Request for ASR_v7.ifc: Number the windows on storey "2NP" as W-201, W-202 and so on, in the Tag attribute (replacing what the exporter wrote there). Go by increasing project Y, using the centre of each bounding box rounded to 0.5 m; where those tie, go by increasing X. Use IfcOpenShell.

First a look at what the model holds.

```python
import ifcopenshell
import ifcopenshell.util.element
import ifcopenshell.util.placement

model = ifcopenshell.open("ASR_v7.ifc")
print(model.schema)
storey = next(s for s in model.by_type("IfcBuildingStorey") if s.Name == "2NP")
windows = [e for e in ifcopenshell.util.element.get_decomposition(storey) if e.is_a("IfcWindow")]
for e in sorted(windows, key=lambda e: e.id()):
    origin = ifcopenshell.util.placement.get_local_placement(e.ObjectPlacement)[:3, 3]
    print(e.id(), e.Tag, e.Name, origin.round(2) + 0.0, sep=" | ")
```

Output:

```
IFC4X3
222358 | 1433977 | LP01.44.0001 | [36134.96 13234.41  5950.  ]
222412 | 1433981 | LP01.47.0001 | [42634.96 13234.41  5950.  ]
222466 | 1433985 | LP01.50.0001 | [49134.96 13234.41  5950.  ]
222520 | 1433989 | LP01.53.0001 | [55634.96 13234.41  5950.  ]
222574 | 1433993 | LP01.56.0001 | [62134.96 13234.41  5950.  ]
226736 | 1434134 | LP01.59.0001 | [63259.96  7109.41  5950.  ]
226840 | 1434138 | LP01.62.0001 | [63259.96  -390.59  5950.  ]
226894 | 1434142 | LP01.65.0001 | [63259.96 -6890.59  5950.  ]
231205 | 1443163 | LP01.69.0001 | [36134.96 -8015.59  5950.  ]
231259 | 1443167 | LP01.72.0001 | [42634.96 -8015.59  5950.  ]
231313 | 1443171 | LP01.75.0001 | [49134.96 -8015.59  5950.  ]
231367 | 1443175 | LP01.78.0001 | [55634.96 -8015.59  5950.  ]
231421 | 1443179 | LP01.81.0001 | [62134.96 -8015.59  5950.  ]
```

```python
import ifcopenshell
import ifcopenshell.geom
import ifcopenshell.util.element
import ifcopenshell.util.shape

model = ifcopenshell.open("ASR_v7.ifc")
settings = ifcopenshell.geom.settings()
settings.set("use-world-coords", True)


def centre(element):
    shape = ifcopenshell.geom.create_shape(settings, element)
    return ifcopenshell.util.shape.get_bbox_centroid(shape.geometry)


storey = next(s for s in model.by_type("IfcBuildingStorey") if s.Name == "2NP")
windows = [e for e in ifcopenshell.util.element.get_decomposition(storey) if e.is_a("IfcWindow")]

# Insertion points can sit at a corner or the storey origin, so sort by the geometry (in metres).
centres = {e: centre(e) for e in windows}
windows.sort(key=lambda e: (round(centres[e][1] / 0.5), centres[e][0]))

for i, e in enumerate(windows, start=1):
    number = f"W-2{i:02d}"
    e.Tag = number
    print(e.id(), number)

model.write("ASR_v7_rev.ifc")
```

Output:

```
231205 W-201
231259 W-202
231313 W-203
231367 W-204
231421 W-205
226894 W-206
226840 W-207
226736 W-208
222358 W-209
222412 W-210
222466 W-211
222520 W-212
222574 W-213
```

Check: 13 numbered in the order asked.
